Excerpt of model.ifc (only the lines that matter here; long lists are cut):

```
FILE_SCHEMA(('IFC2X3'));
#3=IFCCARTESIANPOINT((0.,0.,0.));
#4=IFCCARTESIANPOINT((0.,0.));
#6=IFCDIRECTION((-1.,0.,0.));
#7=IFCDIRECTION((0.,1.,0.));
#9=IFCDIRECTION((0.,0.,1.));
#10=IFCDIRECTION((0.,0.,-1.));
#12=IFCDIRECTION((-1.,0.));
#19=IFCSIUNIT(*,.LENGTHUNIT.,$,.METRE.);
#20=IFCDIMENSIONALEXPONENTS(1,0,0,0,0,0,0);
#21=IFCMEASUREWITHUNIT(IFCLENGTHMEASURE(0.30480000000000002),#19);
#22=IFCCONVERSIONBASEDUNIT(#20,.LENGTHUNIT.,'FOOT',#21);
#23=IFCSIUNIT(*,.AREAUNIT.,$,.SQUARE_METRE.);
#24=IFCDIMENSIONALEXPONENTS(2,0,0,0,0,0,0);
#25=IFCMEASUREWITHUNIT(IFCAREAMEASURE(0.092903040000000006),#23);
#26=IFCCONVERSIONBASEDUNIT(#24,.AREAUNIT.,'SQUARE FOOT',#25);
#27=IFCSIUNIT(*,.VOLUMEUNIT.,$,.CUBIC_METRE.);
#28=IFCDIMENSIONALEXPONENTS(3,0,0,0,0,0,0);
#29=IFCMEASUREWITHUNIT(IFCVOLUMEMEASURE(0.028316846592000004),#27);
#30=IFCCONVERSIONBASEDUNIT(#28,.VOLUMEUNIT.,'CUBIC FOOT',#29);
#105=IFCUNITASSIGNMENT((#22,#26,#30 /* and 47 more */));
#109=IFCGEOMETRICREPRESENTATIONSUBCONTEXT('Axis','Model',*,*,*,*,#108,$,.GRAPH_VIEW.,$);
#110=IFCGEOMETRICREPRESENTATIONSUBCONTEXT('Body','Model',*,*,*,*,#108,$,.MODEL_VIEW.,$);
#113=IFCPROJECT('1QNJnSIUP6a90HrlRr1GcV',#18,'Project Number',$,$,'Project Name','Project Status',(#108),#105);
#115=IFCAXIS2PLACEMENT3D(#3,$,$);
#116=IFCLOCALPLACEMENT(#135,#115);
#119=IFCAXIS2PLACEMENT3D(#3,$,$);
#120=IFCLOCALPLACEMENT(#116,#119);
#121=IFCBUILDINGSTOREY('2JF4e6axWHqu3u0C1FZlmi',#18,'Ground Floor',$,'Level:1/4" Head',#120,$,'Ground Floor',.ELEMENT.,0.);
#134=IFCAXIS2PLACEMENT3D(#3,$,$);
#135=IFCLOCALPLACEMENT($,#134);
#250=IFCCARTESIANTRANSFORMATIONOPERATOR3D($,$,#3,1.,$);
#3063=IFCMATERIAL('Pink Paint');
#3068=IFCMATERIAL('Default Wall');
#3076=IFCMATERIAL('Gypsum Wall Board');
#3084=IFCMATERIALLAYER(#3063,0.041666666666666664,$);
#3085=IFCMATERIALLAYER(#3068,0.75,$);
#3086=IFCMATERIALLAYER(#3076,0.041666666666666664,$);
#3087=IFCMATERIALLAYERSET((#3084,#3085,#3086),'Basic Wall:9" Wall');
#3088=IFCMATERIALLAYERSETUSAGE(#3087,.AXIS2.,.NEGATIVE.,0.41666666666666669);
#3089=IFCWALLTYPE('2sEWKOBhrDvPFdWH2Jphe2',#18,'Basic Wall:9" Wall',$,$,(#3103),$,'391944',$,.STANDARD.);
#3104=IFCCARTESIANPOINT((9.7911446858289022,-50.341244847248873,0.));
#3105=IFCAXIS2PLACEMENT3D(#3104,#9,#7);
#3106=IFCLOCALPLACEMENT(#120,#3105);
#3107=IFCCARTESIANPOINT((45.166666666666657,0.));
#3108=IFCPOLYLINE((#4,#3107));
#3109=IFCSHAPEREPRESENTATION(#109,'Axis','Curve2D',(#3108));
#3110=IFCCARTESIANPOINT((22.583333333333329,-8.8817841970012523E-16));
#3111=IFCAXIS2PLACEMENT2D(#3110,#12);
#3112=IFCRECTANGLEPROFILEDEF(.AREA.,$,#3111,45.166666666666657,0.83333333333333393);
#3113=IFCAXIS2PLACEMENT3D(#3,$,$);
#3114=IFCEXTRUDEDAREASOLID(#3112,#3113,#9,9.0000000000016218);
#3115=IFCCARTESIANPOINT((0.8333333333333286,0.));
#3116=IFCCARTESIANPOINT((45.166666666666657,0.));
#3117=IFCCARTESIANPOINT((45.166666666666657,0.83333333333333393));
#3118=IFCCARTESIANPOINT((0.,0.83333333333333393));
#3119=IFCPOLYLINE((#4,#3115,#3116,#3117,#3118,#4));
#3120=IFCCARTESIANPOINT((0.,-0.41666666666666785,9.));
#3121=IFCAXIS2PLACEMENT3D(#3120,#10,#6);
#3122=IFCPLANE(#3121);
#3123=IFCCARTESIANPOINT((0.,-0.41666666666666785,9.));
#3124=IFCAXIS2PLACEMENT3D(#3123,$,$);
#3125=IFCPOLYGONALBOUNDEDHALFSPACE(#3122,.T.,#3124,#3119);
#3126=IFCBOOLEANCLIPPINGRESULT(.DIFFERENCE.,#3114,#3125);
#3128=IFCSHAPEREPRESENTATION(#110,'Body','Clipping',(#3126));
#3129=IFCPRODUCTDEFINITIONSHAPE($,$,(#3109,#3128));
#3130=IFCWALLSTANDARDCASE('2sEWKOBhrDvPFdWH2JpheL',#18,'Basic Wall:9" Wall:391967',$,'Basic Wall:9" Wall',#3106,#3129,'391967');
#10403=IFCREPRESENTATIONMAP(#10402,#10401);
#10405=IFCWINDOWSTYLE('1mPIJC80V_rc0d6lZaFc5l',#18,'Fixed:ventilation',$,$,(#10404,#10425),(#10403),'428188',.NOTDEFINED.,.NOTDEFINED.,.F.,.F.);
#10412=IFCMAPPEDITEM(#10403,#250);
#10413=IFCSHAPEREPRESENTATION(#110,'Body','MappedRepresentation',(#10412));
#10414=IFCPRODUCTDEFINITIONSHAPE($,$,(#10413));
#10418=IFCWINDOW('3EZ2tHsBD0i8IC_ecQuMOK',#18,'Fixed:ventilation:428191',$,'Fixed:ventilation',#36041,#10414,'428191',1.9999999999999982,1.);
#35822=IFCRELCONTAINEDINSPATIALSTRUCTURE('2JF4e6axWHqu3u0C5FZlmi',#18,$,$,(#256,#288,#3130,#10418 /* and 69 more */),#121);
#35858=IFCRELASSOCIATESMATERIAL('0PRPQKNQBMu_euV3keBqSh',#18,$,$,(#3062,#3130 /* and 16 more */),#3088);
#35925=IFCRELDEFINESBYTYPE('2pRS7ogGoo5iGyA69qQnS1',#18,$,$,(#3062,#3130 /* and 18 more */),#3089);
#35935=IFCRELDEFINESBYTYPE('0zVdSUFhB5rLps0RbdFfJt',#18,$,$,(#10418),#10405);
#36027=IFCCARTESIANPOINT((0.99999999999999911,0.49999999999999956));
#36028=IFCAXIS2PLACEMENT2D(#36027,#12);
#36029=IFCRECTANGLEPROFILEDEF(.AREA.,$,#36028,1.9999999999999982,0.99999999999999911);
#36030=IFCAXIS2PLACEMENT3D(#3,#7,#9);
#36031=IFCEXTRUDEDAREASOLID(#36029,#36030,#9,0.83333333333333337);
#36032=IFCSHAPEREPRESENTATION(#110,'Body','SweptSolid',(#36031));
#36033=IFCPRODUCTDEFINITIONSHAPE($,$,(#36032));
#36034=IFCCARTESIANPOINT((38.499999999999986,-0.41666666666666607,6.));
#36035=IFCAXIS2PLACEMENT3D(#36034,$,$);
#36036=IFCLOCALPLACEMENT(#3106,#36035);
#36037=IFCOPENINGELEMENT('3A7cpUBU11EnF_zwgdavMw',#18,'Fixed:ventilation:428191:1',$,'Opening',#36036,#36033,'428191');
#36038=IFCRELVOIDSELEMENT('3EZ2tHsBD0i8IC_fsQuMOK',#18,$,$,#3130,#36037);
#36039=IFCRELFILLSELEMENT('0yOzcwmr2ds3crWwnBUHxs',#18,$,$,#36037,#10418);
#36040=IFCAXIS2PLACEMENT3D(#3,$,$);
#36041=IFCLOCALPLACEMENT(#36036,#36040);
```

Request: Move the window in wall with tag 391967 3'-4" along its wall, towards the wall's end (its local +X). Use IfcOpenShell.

```python
import ifcopenshell
import ifcopenshell.api.geometry
import ifcopenshell.util.placement
import ifcopenshell.util.unit

model = ifcopenshell.open("model.ifc")
unit_scale = ifcopenshell.util.unit.calculate_unit_scale(model)

window = model.by_guid("3EZ2tHsBD0i8IC_ecQuMOK")
opening = window.FillsVoids[0].RelatingOpeningElement
wall = opening.VoidsElements[0].RelatingBuildingElement

wall_matrix = ifcopenshell.util.placement.get_local_placement(wall.ObjectPlacement)
shift = wall_matrix[:3, 0] * 40 * 0.0254 / unit_scale
before = ifcopenshell.util.placement.get_local_placement(window.ObjectPlacement)[:3, 3].copy()

# The window is placed relative to its opening, so it follows when the opening moves.
matrix = ifcopenshell.util.placement.get_local_placement(opening.ObjectPlacement)
matrix[:3, 3] += shift
ifcopenshell.api.geometry.edit_object_placement(
    model, product=opening, matrix=matrix, is_si=False, should_transform_children=True
)

after = ifcopenshell.util.placement.get_local_placement(window.ObjectPlacement)[:3, 3]
print("window moved by", (after - before).round(3) + 0.0)

model.write("model_updated.ifc")
```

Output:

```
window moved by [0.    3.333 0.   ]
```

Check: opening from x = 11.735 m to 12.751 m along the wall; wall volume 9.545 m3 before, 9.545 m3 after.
